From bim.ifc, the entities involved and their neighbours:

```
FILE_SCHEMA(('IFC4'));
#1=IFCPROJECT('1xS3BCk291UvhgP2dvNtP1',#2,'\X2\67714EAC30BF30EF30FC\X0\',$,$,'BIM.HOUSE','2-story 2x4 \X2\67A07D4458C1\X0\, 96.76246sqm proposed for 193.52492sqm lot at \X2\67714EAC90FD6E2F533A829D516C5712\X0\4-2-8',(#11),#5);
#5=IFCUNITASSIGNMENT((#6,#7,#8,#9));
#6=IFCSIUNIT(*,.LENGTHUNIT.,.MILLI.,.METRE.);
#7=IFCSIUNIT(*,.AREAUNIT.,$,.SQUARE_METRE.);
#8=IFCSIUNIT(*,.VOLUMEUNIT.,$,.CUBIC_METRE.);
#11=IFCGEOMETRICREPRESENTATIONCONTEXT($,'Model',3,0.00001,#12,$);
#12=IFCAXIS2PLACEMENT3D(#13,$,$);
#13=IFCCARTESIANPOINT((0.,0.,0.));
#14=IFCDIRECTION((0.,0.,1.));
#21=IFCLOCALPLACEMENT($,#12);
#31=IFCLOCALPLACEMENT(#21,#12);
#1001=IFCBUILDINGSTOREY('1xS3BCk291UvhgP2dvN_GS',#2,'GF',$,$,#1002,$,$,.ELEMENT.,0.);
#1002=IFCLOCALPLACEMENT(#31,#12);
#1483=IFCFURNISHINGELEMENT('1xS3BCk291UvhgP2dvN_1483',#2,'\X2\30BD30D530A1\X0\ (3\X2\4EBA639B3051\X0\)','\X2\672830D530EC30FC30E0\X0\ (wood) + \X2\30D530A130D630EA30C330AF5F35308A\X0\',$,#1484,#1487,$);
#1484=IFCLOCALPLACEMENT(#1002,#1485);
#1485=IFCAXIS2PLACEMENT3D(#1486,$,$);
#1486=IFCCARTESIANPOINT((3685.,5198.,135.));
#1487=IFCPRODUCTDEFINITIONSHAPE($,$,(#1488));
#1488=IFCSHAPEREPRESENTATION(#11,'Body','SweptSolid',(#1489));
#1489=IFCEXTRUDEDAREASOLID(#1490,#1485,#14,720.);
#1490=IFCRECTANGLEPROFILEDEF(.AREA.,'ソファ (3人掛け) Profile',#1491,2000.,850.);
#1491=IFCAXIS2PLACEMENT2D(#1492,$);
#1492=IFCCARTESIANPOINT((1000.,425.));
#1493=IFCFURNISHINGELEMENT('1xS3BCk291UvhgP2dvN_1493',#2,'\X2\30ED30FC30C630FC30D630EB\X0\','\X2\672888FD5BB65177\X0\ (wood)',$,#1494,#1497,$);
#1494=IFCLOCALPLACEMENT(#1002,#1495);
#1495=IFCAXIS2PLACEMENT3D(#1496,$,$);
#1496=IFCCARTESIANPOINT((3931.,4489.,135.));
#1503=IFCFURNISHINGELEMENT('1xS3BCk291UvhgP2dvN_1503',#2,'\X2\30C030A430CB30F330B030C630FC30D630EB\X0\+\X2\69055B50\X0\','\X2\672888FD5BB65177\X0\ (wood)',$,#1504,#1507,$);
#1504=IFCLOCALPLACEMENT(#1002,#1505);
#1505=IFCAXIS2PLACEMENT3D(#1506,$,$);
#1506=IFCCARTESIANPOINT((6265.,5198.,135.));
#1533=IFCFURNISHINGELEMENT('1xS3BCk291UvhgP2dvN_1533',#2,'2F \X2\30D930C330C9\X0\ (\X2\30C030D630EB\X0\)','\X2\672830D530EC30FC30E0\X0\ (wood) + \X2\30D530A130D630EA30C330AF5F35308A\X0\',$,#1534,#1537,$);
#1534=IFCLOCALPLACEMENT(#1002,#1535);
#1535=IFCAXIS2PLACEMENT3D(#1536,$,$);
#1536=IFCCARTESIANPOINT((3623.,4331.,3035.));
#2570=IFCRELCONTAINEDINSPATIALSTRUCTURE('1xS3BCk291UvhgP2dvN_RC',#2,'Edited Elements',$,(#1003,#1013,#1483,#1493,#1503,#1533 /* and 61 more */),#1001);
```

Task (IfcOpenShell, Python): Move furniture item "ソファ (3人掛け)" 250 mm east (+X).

```python
import ifcopenshell
import ifcopenshell.api.geometry
import ifcopenshell.util.placement

model = ifcopenshell.open("bim.ifc")

item = model.by_guid("1xS3BCk291UvhgP2dvN_1483")
matrix = ifcopenshell.util.placement.get_local_placement(item.ObjectPlacement)
matrix[0, 3] += 250.0
ifcopenshell.api.geometry.edit_object_placement(model, product=item, matrix=matrix, is_si=False)

print(ifcopenshell.util.placement.get_local_placement(item.ObjectPlacement).round(3) + 0.0)

model.write("bim-out.ifc")
```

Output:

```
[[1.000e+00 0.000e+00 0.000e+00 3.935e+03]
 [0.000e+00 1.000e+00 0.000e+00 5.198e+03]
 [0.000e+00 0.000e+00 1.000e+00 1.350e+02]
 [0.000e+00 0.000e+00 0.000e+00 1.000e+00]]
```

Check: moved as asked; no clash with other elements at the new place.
